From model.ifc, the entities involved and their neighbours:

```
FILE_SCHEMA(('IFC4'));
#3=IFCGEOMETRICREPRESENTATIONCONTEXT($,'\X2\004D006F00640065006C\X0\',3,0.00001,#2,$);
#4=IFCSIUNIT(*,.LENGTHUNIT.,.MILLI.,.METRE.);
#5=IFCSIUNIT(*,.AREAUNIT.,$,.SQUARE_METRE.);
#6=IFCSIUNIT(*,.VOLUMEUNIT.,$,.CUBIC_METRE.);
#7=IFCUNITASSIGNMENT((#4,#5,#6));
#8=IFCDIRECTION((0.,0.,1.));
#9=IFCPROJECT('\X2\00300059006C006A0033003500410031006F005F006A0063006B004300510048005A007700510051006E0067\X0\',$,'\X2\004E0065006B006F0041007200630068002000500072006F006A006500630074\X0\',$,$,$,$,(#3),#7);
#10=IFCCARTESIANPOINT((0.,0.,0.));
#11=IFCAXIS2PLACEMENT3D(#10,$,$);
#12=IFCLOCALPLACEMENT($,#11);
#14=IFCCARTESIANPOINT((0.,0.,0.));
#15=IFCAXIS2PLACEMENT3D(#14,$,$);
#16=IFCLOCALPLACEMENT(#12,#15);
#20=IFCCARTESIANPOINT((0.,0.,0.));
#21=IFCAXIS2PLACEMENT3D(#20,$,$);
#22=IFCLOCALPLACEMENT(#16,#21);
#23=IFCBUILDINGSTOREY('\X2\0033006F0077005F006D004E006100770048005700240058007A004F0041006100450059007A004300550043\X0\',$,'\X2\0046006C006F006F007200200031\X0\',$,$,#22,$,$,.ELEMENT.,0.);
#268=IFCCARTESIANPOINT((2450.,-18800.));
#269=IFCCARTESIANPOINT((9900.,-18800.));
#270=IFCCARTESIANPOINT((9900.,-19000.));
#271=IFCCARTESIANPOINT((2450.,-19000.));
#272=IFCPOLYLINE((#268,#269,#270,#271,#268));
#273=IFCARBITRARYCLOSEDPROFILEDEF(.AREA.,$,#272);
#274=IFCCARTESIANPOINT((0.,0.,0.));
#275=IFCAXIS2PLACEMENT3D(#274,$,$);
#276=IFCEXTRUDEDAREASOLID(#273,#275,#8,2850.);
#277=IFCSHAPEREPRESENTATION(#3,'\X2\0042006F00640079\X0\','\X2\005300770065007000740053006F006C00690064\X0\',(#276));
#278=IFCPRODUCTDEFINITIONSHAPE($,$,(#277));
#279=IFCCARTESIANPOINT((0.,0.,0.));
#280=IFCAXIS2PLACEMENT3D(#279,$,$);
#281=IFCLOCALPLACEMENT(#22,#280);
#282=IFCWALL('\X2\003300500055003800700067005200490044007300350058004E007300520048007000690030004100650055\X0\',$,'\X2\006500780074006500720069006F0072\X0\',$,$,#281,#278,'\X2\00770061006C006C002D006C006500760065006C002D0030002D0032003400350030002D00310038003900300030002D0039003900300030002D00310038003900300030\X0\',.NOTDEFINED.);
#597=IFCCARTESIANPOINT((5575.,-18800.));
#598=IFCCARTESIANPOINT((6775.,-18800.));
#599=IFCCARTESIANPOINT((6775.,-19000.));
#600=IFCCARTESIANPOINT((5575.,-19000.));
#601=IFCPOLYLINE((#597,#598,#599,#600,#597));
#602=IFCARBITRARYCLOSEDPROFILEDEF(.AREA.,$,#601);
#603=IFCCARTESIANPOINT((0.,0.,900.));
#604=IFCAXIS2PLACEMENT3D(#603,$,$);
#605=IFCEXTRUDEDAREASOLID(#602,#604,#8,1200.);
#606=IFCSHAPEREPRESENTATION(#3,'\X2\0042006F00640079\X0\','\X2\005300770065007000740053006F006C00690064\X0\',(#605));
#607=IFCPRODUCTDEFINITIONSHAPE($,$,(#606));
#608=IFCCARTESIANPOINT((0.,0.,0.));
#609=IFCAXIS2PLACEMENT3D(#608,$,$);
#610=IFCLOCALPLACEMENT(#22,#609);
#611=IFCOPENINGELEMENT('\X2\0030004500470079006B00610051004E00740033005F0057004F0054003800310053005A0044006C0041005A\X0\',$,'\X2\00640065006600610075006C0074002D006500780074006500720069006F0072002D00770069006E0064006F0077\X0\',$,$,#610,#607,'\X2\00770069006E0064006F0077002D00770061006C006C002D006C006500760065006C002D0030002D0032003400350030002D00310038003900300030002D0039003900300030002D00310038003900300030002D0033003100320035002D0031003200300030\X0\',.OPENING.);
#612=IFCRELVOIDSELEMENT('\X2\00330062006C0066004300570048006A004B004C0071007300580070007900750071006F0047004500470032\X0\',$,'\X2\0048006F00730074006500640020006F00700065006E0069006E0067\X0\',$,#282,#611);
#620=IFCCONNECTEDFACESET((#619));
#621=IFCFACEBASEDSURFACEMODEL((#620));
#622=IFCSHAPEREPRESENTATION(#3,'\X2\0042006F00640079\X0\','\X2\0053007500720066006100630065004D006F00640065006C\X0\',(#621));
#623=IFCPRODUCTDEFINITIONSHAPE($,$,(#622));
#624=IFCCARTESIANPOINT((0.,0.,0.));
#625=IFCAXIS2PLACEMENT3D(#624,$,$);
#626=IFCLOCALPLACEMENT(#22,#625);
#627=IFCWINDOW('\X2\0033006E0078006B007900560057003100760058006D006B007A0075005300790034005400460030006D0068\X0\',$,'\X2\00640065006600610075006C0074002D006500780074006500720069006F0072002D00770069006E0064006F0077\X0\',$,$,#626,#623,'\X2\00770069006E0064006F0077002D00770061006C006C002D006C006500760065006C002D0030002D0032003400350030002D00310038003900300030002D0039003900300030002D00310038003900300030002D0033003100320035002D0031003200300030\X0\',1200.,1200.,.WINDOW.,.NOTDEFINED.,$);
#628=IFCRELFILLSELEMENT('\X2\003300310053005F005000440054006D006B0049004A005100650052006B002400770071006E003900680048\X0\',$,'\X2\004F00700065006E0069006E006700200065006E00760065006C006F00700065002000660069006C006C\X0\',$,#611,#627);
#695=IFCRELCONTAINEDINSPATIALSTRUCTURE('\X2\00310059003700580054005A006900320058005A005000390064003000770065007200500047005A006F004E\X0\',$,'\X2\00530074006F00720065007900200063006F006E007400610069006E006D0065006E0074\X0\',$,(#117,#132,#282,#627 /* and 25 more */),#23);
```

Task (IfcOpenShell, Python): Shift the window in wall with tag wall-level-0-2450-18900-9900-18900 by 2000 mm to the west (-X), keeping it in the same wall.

```python
import ifcopenshell
import ifcopenshell.api.geometry
import ifcopenshell.util.placement
import ifcopenshell.util.unit

model = ifcopenshell.open("model.ifc")
unit_scale = ifcopenshell.util.unit.calculate_unit_scale(model)

window = model.by_guid("3nxkyVW1vXmkzuSy4TF0mh")
opening = window.FillsVoids[0].RelatingOpeningElement
wall = opening.VoidsElements[0].RelatingBuildingElement

wall_matrix = ifcopenshell.util.placement.get_local_placement(wall.ObjectPlacement)
shift = wall_matrix[:3, 0] * -2 / unit_scale
before = ifcopenshell.util.placement.get_local_placement(window.ObjectPlacement)[:3, 3].copy()

# The window is not placed relative to its opening, so move both.
for product in (opening, window):
    matrix = ifcopenshell.util.placement.get_local_placement(product.ObjectPlacement)
    matrix[:3, 3] += shift
    ifcopenshell.api.geometry.edit_object_placement(model, product=product, matrix=matrix, is_si=False)

after = ifcopenshell.util.placement.get_local_placement(window.ObjectPlacement)[:3, 3]
print("window moved by", (after - before).round(3) + 0.0)

model.write("model_rev.ifc")
```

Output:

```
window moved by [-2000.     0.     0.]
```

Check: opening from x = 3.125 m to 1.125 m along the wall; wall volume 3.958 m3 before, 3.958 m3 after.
